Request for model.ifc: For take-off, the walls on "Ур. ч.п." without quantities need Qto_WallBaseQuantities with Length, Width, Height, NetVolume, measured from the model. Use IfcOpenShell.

First a look at what the model holds.

```python
import ifcopenshell
import ifcopenshell.util.element
import ifcopenshell.util.unit

model = ifcopenshell.open("model.ifc")
print(model.schema)
for unit_type in ("LENGTHUNIT", "AREAUNIT", "VOLUMEUNIT"):
    print(unit_type, ifcopenshell.util.unit.calculate_unit_scale(model, unit_type))
storey = next(s for s in model.by_type("IfcBuildingStorey") if s.Name == "Ур. ч.п.")
walls = [e for e in ifcopenshell.util.element.get_decomposition(storey) if e.is_a("IfcWall")]
for e in sorted(walls, key=lambda e: e.id()):
    print(e.id(), e.is_a(), e.Name, list(ifcopenshell.util.element.get_psets(e, qtos_only=True)), sep=" | ")
```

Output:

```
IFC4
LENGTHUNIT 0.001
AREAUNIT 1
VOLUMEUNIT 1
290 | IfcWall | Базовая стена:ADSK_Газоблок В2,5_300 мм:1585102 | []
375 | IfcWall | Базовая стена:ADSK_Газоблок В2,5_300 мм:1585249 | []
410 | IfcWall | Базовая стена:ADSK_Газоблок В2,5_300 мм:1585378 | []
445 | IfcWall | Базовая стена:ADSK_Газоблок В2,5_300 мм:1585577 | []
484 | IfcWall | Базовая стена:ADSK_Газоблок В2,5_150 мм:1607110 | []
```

```python
import ifcopenshell
import ifcopenshell.api.pset
import ifcopenshell.geom
import ifcopenshell.util.element
import ifcopenshell.util.shape
import ifcopenshell.util.unit

model = ifcopenshell.open("model.ifc")
unit_scale = ifcopenshell.util.unit.calculate_unit_scale(model)
volume_scale = ifcopenshell.util.unit.calculate_unit_scale(model, "VOLUMEUNIT")
settings = ifcopenshell.geom.settings()

storey = next(s for s in model.by_type("IfcBuildingStorey") if s.Name == "Ур. ч.п.")
walls = [e for e in ifcopenshell.util.element.get_decomposition(storey) if e.is_a("IfcWall")]

for e in sorted(walls, key=lambda e: e.id()):
    if ifcopenshell.util.element.get_psets(e, qtos_only=True, should_inherit=False):
        continue
    # Geometry comes back in metres, in the element's own axes.
    shape = ifcopenshell.geom.create_shape(settings, e)
    values = {
        "Length": ifcopenshell.util.shape.get_x(shape.geometry) / unit_scale,
        "Width": ifcopenshell.util.shape.get_y(shape.geometry) / unit_scale,
        "Height": ifcopenshell.util.shape.get_z(shape.geometry) / unit_scale,
        "NetVolume": ifcopenshell.util.shape.get_volume(shape.geometry) / volume_scale,
    }
    qto = ifcopenshell.api.pset.add_qto(model, product=e, name="Qto_WallBaseQuantities")
    ifcopenshell.api.pset.edit_qto(model, qto=qto, properties=values)
    print(e.id(), {k: round(v, 3) for k, v in values.items()})

model.write("model_v2.ifc")
```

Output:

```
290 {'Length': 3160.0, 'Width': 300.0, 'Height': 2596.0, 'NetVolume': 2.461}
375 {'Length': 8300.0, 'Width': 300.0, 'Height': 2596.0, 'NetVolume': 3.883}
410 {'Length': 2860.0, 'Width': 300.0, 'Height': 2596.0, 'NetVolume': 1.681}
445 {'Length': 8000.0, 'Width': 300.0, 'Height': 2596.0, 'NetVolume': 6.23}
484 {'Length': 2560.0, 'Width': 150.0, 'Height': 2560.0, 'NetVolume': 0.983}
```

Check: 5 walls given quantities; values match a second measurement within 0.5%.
